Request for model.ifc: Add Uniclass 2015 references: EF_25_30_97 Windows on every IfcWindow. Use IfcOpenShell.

First a look at what the model holds.

```python
import ifcopenshell

model = ifcopenshell.open("model.ifc")
print(model.schema)
print("classifications:", [c.Name for c in model.by_type("IfcClassification")])
for ifc_class in ("IfcDoor", "IfcRoof", "IfcStair", "IfcWall", "IfcWindow"):
    print(ifc_class, len(model.by_type(ifc_class)))
```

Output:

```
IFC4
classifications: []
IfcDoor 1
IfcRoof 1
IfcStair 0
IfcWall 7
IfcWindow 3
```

```python
import ifcopenshell
import ifcopenshell.api.classification

model = ifcopenshell.open("model.ifc")

system = ifcopenshell.api.classification.add_classification(model, classification="Uniclass 2015")

codes = {
    "IfcWindow": ("EF_25_30_97", "Windows"),
}
for ifc_class, (code, name) in codes.items():
    products = model.by_type(ifc_class)
    ifcopenshell.api.classification.add_reference(
        model, products=products, classification=system, identification=code, name=name
    )
    print(code, len(products))

model.write("model-out.ifc")
```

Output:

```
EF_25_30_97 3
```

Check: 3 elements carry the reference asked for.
